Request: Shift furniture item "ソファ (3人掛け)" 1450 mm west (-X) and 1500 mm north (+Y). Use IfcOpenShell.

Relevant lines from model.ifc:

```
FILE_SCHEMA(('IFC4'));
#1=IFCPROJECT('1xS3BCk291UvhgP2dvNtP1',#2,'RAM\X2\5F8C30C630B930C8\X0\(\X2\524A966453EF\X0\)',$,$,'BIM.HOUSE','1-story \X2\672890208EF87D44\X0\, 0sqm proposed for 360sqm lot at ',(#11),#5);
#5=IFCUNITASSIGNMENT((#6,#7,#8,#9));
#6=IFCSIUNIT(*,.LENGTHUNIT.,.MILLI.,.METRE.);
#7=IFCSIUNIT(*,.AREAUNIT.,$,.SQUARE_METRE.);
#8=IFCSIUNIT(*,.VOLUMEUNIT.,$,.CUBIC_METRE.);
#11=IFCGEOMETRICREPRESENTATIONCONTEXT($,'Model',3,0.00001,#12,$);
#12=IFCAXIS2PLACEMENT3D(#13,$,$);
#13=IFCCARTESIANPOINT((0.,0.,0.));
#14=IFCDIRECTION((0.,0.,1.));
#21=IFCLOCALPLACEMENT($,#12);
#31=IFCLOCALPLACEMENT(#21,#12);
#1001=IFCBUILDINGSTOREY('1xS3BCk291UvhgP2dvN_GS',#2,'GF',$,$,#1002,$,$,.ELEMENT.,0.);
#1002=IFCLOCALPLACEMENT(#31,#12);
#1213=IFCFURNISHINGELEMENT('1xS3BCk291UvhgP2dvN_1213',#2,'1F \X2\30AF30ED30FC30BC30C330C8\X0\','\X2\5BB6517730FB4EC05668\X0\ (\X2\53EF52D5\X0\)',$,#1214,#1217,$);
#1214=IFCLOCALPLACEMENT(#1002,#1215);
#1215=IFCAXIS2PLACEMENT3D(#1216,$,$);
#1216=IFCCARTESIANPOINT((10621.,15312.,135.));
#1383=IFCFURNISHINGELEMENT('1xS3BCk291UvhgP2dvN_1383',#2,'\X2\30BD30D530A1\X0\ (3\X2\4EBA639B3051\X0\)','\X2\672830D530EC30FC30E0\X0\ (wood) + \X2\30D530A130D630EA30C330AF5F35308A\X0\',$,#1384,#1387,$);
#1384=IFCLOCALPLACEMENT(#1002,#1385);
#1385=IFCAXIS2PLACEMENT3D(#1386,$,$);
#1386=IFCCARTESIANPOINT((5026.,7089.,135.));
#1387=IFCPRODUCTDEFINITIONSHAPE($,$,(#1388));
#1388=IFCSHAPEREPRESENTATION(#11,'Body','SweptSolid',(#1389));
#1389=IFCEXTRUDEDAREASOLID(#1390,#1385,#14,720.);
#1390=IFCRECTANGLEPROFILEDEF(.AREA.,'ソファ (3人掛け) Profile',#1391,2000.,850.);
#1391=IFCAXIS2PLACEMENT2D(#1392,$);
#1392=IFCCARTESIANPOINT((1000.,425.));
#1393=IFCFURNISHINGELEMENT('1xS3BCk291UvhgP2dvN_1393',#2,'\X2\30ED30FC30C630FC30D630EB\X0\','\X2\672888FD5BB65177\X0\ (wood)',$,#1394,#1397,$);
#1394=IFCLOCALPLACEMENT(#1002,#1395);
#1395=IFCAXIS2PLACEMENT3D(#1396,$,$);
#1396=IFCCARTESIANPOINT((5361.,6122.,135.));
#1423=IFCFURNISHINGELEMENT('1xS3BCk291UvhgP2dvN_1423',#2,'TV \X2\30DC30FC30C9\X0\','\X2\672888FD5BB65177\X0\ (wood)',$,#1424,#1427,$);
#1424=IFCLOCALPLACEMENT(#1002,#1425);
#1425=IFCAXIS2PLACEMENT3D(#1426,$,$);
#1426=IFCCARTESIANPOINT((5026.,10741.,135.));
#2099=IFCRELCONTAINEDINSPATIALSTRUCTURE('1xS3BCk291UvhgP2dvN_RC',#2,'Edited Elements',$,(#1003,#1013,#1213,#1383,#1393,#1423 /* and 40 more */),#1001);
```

```python
import ifcopenshell
import ifcopenshell.api.geometry
import ifcopenshell.util.placement

model = ifcopenshell.open("model.ifc")

item = model.by_id(1383)
matrix = ifcopenshell.util.placement.get_local_placement(item.ObjectPlacement)
matrix[0, 3] -= 1450.0
matrix[1, 3] += 1500.0
ifcopenshell.api.geometry.edit_object_placement(model, product=item, matrix=matrix, is_si=False)

print(ifcopenshell.util.placement.get_local_placement(item.ObjectPlacement).round(3) + 0.0)

model.write("model-out.ifc")
```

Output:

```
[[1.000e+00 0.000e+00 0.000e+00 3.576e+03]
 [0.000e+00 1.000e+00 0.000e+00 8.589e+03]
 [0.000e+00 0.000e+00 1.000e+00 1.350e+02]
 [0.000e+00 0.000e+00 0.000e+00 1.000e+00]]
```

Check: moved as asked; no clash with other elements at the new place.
